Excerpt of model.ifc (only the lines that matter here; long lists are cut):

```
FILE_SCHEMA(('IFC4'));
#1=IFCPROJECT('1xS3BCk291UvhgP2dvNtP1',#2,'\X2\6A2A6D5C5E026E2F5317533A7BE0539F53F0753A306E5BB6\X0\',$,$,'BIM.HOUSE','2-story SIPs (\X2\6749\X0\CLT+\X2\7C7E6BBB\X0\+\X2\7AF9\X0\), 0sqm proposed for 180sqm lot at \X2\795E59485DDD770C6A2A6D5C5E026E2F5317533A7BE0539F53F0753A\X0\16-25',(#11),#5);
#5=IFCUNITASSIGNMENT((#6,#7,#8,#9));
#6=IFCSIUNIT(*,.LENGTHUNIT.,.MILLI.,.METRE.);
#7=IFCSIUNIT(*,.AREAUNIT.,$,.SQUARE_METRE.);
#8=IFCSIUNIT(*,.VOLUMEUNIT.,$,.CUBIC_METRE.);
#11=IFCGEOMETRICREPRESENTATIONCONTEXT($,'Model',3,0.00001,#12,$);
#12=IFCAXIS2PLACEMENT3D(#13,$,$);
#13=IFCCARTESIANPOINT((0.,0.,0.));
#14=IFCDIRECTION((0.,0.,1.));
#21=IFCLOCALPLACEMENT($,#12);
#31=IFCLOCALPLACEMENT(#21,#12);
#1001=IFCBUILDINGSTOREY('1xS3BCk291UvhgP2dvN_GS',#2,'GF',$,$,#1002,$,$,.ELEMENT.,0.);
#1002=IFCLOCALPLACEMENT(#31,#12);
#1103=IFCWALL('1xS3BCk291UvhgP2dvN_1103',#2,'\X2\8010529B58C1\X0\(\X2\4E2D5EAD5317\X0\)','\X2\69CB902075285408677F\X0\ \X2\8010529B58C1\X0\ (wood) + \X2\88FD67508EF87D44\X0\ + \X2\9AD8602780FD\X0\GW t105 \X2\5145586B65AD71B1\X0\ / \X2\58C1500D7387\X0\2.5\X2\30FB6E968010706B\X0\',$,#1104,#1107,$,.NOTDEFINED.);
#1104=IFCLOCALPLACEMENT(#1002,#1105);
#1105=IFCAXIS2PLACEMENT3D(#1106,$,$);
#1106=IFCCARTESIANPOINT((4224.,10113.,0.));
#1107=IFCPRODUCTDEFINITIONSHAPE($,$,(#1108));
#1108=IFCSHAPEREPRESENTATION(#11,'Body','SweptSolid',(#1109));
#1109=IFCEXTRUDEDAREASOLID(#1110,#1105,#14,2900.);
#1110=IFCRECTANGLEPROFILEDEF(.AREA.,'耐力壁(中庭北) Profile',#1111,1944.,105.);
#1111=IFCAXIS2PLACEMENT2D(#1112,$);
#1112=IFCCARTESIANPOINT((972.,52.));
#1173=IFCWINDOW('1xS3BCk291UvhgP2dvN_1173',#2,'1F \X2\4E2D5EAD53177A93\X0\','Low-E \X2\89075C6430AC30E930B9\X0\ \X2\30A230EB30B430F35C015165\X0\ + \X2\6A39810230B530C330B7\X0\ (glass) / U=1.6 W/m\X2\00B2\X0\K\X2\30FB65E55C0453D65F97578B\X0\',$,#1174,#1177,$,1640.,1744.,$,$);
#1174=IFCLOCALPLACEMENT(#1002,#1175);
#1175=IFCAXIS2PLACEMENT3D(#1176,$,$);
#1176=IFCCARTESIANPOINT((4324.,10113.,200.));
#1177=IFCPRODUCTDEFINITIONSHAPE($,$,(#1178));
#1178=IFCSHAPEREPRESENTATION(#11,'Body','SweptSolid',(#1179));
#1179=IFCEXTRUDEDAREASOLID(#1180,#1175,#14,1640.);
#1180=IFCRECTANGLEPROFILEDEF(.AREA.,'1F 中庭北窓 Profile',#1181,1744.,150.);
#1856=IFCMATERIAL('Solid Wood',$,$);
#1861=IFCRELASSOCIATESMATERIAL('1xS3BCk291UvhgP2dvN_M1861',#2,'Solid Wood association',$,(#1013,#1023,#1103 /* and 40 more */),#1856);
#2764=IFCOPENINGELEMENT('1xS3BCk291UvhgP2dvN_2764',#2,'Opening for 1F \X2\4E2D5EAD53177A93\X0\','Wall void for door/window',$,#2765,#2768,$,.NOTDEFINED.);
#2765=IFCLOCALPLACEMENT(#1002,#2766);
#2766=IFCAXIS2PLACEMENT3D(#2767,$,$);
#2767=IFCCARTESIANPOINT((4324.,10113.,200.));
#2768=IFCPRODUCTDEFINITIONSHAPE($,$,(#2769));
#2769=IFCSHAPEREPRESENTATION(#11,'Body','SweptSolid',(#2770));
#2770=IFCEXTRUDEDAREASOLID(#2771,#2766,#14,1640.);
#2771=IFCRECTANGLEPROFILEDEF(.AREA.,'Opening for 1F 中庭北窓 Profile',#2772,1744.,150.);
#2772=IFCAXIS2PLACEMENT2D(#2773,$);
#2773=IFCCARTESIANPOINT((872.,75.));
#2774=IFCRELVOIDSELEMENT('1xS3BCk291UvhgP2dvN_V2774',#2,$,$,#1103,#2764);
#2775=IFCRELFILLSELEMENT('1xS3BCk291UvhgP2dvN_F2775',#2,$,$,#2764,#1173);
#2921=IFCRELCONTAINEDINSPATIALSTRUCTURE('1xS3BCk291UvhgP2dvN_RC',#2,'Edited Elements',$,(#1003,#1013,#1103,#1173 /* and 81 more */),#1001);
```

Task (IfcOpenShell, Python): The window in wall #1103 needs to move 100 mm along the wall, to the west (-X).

```python
import ifcopenshell
import ifcopenshell.api.geometry
import ifcopenshell.util.placement
import ifcopenshell.util.unit

model = ifcopenshell.open("model.ifc")
unit_scale = ifcopenshell.util.unit.calculate_unit_scale(model)

window = model.by_guid("1xS3BCk291UvhgP2dvN_1173")
opening = window.FillsVoids[0].RelatingOpeningElement
wall = opening.VoidsElements[0].RelatingBuildingElement

wall_matrix = ifcopenshell.util.placement.get_local_placement(wall.ObjectPlacement)
shift = wall_matrix[:3, 0] * -0.1 / unit_scale
before = ifcopenshell.util.placement.get_local_placement(window.ObjectPlacement)[:3, 3].copy()

# The window is not placed relative to its opening, so move both.
for product in (opening, window):
    matrix = ifcopenshell.util.placement.get_local_placement(product.ObjectPlacement)
    matrix[:3, 3] += shift
    ifcopenshell.api.geometry.edit_object_placement(model, product=product, matrix=matrix, is_si=False)

after = ifcopenshell.util.placement.get_local_placement(window.ObjectPlacement)[:3, 3]
print("window moved by", (after - before).round(3) + 0.0)

model.write("model_rev.ifc")
```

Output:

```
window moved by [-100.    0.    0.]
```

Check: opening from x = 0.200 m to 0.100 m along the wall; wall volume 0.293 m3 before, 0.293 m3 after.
